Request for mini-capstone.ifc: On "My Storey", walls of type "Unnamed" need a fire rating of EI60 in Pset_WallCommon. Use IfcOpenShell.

First a look at what the model holds.

```python
import ifcopenshell
import ifcopenshell.util.element

model = ifcopenshell.open("mini-capstone.ifc")
print(model.schema)
storey = next(s for s in model.by_type("IfcBuildingStorey") if s.Name == "My Storey")
walls = [e for e in ifcopenshell.util.element.get_decomposition(storey) if e.is_a("IfcWall")]
seen = {}
for e in walls:
    element_type = ifcopenshell.util.element.get_type(e)
    key = (element_type.Name if element_type != e and element_type else None, ifcopenshell.util.element.get_pset(e, "Pset_WallCommon", "FireRating"))
    seen[key] = seen.get(key, 0) + 1
for (name, value), count in sorted(seen.items(), key=str):
    print(count, "x", name, "|", value)
```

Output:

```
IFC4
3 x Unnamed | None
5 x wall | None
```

```python
import ifcopenshell
import ifcopenshell.api.pset
import ifcopenshell.util.element

model = ifcopenshell.open("mini-capstone.ifc")

storey = next(s for s in model.by_type("IfcBuildingStorey") if s.Name == "My Storey")
walls = [e for e in ifcopenshell.util.element.get_decomposition(storey) if e.is_a("IfcWall")]

count = 0
for e in walls:
    element_type = ifcopenshell.util.element.get_type(e)
    if element_type in (None, e) or element_type.Name != "Unnamed":
        continue
    # add_pset returns the element's existing set when there is one.
    pset = ifcopenshell.api.pset.add_pset(model, product=e, name="Pset_WallCommon")
    ifcopenshell.api.pset.edit_pset(model, pset=pset, properties={"FireRating": "EI60"})
    count += 1

print(count, "walls updated")

model.write("mini-capstone_edited.ifc")
```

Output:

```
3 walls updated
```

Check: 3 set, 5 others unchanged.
